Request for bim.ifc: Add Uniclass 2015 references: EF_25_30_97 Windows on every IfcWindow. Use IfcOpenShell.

First a look at what the model holds.

```python
import ifcopenshell

model = ifcopenshell.open("bim.ifc")
print(model.schema)
print("classifications:", [c.Name for c in model.by_type("IfcClassification")])
for ifc_class in ("IfcDoor", "IfcRoof", "IfcStair", "IfcWall", "IfcWindow"):
    print(ifc_class, len(model.by_type(ifc_class)))
```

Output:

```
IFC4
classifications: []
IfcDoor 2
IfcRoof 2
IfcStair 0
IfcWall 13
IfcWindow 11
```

```python
import ifcopenshell
import ifcopenshell.api.classification

model = ifcopenshell.open("bim.ifc")

system = ifcopenshell.api.classification.add_classification(model, classification="Uniclass 2015")

codes = {
    "IfcWindow": ("EF_25_30_97", "Windows"),
}
for ifc_class, (code, name) in codes.items():
    products = model.by_type(ifc_class)
    ifcopenshell.api.classification.add_reference(
        model, products=products, classification=system, identification=code, name=name
    )
    print(code, len(products))

model.write("bim_v2.ifc")
```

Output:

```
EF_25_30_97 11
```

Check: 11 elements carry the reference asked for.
